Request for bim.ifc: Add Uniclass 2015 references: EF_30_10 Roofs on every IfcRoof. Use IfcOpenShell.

First a look at what the model holds.

```python
import ifcopenshell

model = ifcopenshell.open("bim.ifc")
print(model.schema)
print("classifications:", [c.Name for c in model.by_type("IfcClassification")])
for ifc_class in ("IfcDoor", "IfcRoof", "IfcStair", "IfcWall", "IfcWindow"):
    print(ifc_class, len(model.by_type(ifc_class)))
```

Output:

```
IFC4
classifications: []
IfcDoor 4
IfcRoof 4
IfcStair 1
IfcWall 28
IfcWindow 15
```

```python
import ifcopenshell
import ifcopenshell.api.classification

model = ifcopenshell.open("bim.ifc")

system = ifcopenshell.api.classification.add_classification(model, classification="Uniclass 2015")

codes = {
    "IfcRoof": ("EF_30_10", "Roofs"),
}
for ifc_class, (code, name) in codes.items():
    products = model.by_type(ifc_class)
    ifcopenshell.api.classification.add_reference(
        model, products=products, classification=system, identification=code, name=name
    )
    print(code, len(products))

model.write("bim_updated.ifc")
```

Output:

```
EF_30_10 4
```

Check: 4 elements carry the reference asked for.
